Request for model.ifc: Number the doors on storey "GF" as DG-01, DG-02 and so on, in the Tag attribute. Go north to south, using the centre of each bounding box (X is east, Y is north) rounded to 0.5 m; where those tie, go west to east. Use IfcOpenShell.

First a look at what the model holds.

```python
import ifcopenshell
import ifcopenshell.util.element
import ifcopenshell.util.placement

model = ifcopenshell.open("model.ifc")
print(model.schema)
storey = next(s for s in model.by_type("IfcBuildingStorey") if s.Name == "GF")
doors = [e for e in ifcopenshell.util.element.get_decomposition(storey) if e.is_a("IfcDoor")]
for e in sorted(doors, key=lambda e: e.id()):
    origin = ifcopenshell.util.placement.get_local_placement(e.ObjectPlacement)[:3, 3]
    print(e.id(), e.Tag, e.Name, origin.round(2) + 0.0, sep=" | ")
```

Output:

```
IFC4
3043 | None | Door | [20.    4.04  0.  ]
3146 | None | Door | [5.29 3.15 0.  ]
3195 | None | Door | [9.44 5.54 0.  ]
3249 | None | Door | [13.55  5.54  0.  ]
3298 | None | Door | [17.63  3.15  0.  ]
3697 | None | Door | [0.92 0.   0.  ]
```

```python
import ifcopenshell
import ifcopenshell.geom
import ifcopenshell.util.element
import ifcopenshell.util.shape

model = ifcopenshell.open("model.ifc")
settings = ifcopenshell.geom.settings()
settings.set("use-world-coords", True)


def centre(element):
    shape = ifcopenshell.geom.create_shape(settings, element)
    return ifcopenshell.util.shape.get_bbox_centroid(shape.geometry)


storey = next(s for s in model.by_type("IfcBuildingStorey") if s.Name == "GF")
doors = [e for e in ifcopenshell.util.element.get_decomposition(storey) if e.is_a("IfcDoor")]

# Insertion points can sit at a corner or the storey origin, so sort by the geometry (in metres).
centres = {e: centre(e) for e in doors}
doors.sort(key=lambda e: (-round(centres[e][1] / 0.5), centres[e][0]))

for i, e in enumerate(doors, start=1):
    number = f"DG-{i:02d}"
    e.Tag = number
    print(e.id(), number)

model.write("model_updated.ifc")
```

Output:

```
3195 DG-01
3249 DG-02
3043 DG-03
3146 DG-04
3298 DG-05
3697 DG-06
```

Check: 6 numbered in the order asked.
